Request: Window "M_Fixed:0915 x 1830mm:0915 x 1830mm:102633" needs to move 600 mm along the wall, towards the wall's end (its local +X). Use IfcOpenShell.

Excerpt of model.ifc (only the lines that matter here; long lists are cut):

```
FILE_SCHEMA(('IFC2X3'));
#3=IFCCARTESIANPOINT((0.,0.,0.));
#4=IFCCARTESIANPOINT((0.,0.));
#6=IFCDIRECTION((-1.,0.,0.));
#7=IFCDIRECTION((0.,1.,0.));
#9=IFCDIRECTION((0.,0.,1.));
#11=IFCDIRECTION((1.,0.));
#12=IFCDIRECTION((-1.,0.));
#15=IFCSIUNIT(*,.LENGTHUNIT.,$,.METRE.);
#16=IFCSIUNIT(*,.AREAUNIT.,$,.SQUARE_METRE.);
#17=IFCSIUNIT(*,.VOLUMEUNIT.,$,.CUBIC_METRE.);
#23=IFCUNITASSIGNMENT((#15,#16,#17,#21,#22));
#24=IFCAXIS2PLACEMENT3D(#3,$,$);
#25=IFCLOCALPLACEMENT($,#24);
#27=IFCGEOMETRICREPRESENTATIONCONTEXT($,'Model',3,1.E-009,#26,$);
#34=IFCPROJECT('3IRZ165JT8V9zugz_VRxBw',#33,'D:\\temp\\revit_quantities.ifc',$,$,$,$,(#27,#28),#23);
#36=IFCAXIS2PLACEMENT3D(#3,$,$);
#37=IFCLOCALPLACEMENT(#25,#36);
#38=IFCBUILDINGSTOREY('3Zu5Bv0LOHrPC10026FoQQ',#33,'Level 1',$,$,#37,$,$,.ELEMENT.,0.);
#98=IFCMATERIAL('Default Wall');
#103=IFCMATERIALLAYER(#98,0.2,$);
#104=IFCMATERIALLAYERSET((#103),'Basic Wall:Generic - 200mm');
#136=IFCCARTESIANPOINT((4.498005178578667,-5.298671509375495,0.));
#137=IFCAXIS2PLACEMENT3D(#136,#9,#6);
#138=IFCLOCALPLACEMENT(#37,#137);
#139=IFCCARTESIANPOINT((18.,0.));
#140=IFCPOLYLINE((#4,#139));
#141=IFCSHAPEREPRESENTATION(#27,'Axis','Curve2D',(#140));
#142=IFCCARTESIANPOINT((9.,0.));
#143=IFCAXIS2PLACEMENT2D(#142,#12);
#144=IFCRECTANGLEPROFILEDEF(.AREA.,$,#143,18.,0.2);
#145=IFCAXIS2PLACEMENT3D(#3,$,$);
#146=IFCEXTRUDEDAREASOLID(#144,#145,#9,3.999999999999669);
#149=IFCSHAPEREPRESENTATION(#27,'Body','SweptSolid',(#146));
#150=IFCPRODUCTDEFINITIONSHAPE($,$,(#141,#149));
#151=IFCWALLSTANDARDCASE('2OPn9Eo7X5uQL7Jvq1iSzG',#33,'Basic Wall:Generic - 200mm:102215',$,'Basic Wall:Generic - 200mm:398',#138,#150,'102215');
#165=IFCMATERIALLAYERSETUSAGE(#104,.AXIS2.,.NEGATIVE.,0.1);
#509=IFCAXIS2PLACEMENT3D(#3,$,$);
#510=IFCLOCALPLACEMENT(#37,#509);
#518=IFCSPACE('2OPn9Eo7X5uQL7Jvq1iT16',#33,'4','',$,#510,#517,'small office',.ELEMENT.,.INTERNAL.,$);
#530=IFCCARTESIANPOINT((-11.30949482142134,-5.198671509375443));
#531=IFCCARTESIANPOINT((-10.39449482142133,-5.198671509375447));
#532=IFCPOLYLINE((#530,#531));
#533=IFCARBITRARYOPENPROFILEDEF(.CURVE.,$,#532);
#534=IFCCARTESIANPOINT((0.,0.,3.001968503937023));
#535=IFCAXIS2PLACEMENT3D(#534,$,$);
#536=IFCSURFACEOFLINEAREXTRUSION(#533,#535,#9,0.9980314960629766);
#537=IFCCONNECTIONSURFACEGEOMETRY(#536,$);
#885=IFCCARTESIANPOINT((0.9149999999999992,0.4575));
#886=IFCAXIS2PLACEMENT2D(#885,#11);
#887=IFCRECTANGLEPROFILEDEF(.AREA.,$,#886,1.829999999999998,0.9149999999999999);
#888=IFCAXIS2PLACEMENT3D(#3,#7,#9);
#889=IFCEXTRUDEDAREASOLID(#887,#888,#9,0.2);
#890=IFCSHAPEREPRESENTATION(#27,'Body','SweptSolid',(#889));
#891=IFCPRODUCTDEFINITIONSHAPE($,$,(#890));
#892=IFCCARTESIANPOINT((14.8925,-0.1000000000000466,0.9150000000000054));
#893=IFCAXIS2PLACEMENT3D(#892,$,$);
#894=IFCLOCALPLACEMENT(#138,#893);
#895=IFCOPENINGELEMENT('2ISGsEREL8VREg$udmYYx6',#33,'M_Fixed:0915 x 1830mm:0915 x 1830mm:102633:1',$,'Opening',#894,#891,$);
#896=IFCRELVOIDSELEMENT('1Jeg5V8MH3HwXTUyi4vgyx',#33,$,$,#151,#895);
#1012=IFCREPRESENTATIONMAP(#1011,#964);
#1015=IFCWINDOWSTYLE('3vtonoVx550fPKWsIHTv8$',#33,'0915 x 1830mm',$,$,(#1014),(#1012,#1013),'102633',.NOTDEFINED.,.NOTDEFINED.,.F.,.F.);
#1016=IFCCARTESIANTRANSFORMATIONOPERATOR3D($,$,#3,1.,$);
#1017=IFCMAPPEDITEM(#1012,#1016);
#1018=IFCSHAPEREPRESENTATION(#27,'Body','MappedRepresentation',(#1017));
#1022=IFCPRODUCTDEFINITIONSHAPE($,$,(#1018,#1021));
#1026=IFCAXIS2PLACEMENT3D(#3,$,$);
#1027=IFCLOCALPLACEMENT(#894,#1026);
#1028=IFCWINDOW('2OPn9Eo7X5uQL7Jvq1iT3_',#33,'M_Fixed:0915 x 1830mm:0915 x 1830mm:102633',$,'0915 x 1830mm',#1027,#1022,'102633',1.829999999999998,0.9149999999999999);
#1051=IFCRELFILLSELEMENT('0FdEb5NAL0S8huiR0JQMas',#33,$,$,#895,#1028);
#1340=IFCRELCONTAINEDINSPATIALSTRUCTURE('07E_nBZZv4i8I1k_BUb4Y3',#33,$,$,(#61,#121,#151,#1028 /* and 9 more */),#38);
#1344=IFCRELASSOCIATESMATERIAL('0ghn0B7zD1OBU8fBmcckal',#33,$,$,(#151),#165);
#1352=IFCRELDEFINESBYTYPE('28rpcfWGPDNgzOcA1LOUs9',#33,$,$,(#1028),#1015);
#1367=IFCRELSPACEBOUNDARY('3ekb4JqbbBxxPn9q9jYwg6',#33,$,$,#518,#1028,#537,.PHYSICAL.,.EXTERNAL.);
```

```python
import numpy as np
import ifcopenshell
import ifcopenshell.api.geometry
import ifcopenshell.util.placement

model = ifcopenshell.open("model.ifc")

window = model.by_guid("2OPn9Eo7X5uQL7Jvq1iT3_")
opening = window.FillsVoids[0].RelatingOpeningElement
wall = opening.VoidsElements[0].RelatingBuildingElement

wall_matrix = ifcopenshell.util.placement.get_local_placement(wall.ObjectPlacement)
shift = wall_matrix[:3, 0] * 0.6
before = ifcopenshell.util.placement.get_local_placement(window.ObjectPlacement)[:3, 3].copy()

# The window is placed relative to its opening, so it follows when the opening moves.
matrix = ifcopenshell.util.placement.get_local_placement(opening.ObjectPlacement)
matrix[:3, 3] += shift
ifcopenshell.api.geometry.edit_object_placement(
    model, product=opening, matrix=matrix, is_si=False, should_transform_children=True
)

# Space boundary surfaces are stored in each space's coordinates; move them too.
for rel in window.ProvidesBoundaries:
    if not rel.ConnectionGeometry:
        continue
    surface = rel.ConnectionGeometry.SurfaceOnRelatingElement
    space_matrix = ifcopenshell.util.placement.get_local_placement(rel.RelatingSpace.ObjectPlacement)
    point = np.array(surface.Position.Location.Coordinates) + space_matrix[:3, :3].T @ shift
    surface.Position = model.createIfcAxis2Placement3D(
        model.createIfcCartesianPoint(point.tolist()), surface.Position.Axis, surface.Position.RefDirection
    )

after = ifcopenshell.util.placement.get_local_placement(window.ObjectPlacement)[:3, 3]
print("window moved by", (after - before).round(3) + 0.0)

model.write("model_edited.ifc")
```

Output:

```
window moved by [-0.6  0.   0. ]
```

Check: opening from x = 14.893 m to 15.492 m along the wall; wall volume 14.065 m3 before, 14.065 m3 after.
